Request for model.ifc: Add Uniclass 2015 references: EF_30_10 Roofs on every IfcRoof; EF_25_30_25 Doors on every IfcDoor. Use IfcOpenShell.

First a look at what the model holds.

```python
import ifcopenshell

model = ifcopenshell.open("model.ifc")
print(model.schema)
print("classifications:", [c.Name for c in model.by_type("IfcClassification")])
for ifc_class in ("IfcDoor", "IfcRoof", "IfcStair", "IfcWall", "IfcWindow"):
    print(ifc_class, len(model.by_type(ifc_class)))
```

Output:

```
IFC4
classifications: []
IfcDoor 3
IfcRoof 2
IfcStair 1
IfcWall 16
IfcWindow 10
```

```python
import ifcopenshell
import ifcopenshell.api.classification

model = ifcopenshell.open("model.ifc")

system = ifcopenshell.api.classification.add_classification(model, classification="Uniclass 2015")

codes = {
    "IfcRoof": ("EF_30_10", "Roofs"),
    "IfcDoor": ("EF_25_30_25", "Doors"),
}
for ifc_class, (code, name) in codes.items():
    products = model.by_type(ifc_class)
    ifcopenshell.api.classification.add_reference(
        model, products=products, classification=system, identification=code, name=name
    )
    print(code, len(products))

model.write("model-out.ifc")
```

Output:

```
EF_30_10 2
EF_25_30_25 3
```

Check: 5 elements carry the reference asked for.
